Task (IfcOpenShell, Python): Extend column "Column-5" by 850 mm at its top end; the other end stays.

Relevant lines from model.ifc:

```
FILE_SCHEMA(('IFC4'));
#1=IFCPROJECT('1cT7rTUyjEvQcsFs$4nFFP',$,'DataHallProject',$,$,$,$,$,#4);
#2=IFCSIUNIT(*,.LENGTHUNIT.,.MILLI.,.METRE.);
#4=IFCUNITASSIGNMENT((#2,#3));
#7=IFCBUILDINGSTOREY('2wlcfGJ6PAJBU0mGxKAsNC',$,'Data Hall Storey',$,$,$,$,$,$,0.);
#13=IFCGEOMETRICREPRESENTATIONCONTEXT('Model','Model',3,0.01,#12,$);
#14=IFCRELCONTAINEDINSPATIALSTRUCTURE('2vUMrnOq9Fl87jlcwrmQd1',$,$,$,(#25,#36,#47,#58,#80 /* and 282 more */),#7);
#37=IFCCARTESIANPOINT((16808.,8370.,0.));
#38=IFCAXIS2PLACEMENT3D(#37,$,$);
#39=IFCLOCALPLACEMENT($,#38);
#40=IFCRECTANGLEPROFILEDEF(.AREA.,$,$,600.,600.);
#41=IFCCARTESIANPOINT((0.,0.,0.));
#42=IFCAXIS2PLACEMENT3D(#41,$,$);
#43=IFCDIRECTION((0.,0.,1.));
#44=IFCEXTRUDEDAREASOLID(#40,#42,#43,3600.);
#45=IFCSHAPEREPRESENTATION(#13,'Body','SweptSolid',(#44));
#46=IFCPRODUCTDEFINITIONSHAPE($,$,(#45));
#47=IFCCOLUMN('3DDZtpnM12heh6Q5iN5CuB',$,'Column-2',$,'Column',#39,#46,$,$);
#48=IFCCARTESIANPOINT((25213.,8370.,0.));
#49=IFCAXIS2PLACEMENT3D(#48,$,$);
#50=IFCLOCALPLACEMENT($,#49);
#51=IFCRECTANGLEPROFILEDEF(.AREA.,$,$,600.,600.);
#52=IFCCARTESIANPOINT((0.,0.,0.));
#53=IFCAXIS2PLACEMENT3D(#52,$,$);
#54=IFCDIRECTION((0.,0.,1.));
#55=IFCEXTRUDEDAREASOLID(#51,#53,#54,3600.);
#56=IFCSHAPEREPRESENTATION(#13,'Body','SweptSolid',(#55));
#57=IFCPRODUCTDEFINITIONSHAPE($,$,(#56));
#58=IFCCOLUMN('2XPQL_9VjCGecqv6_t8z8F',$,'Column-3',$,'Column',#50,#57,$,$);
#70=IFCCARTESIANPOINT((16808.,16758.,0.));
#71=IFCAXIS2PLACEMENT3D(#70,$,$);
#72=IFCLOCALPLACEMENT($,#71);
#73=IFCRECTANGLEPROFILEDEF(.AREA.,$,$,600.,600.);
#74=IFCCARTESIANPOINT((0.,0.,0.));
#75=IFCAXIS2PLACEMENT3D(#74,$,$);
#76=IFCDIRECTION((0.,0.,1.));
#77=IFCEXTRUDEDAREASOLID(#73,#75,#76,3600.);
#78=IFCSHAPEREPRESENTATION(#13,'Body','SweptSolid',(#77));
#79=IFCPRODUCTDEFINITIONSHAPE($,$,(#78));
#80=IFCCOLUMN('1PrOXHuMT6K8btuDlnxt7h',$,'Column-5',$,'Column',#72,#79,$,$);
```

```python
import ifcopenshell

model = ifcopenshell.open("model.ifc")

member = model.by_id(80)
change = 850.0

# The extrusion runs towards the end named, so only its depth changes.
body = next(r for r in member.Representation.Representations if r.RepresentationIdentifier == "Body")
solid = body.Items[0]
old_length = solid.Depth
solid.Depth += change

print(f"length {old_length:g} -> {solid.Depth:g}")

model.write("model_rev.ifc")
```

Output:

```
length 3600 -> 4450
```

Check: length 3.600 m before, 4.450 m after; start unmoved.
